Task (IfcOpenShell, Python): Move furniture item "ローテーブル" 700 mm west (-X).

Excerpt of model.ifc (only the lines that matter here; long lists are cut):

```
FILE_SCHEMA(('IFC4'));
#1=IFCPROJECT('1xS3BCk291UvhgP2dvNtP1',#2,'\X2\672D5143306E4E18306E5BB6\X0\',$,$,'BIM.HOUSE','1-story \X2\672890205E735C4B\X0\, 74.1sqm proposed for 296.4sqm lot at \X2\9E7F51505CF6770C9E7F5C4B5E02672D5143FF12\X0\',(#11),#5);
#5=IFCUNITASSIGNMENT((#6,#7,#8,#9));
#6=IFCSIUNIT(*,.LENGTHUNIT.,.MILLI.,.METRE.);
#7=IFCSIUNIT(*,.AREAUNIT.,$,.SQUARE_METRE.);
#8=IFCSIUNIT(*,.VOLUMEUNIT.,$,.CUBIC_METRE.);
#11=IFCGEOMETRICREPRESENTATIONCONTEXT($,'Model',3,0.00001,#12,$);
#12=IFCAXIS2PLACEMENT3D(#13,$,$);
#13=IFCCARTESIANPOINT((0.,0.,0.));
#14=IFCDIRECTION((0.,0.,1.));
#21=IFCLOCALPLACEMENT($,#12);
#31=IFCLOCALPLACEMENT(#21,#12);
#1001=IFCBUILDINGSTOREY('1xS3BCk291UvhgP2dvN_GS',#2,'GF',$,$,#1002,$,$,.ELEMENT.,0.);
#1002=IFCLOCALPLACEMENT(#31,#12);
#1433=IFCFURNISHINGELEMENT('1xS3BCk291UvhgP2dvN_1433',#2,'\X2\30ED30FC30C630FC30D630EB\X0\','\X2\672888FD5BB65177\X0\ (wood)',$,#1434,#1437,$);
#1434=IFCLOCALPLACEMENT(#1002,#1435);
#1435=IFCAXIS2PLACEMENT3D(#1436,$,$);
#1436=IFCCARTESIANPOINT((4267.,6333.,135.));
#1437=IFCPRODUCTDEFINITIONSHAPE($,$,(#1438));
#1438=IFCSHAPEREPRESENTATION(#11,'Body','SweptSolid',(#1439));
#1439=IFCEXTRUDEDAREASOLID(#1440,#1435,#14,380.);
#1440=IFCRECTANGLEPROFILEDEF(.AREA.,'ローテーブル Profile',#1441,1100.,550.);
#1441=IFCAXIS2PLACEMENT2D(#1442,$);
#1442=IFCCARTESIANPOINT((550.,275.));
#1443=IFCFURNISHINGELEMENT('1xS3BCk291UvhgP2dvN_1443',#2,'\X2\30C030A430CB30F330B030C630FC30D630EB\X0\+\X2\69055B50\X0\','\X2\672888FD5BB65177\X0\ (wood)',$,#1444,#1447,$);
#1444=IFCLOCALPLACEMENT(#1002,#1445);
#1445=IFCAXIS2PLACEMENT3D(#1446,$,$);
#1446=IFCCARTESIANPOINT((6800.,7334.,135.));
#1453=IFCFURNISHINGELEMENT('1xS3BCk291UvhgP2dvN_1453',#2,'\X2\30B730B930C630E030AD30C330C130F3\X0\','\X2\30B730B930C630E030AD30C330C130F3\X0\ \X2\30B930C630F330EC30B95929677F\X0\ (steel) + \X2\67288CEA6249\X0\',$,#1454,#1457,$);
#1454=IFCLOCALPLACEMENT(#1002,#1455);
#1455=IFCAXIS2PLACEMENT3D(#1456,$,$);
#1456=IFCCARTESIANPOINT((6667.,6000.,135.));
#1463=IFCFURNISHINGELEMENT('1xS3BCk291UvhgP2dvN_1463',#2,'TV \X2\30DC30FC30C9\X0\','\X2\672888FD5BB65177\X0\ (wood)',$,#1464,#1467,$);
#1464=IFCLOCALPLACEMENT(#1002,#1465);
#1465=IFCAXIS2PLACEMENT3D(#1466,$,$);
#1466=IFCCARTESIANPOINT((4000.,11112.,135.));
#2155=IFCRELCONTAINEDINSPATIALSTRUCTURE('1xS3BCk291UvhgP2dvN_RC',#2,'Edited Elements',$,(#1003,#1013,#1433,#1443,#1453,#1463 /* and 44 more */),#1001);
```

```python
import ifcopenshell
import ifcopenshell.api.geometry
import ifcopenshell.util.placement
import ifcopenshell.util.unit

model = ifcopenshell.open("model.ifc")
unit_scale = ifcopenshell.util.unit.calculate_unit_scale(model)

item = model.by_guid("1xS3BCk291UvhgP2dvN_1433")
matrix = ifcopenshell.util.placement.get_local_placement(item.ObjectPlacement)
matrix[0, 3] -= 0.7 / unit_scale
ifcopenshell.api.geometry.edit_object_placement(model, product=item, matrix=matrix, is_si=False)

print(ifcopenshell.util.placement.get_local_placement(item.ObjectPlacement).round(3) + 0.0)

model.write("model_v2.ifc")
```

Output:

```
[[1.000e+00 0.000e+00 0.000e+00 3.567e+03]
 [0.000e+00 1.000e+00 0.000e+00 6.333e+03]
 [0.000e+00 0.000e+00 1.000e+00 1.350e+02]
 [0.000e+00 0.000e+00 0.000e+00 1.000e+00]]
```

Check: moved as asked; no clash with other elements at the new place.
